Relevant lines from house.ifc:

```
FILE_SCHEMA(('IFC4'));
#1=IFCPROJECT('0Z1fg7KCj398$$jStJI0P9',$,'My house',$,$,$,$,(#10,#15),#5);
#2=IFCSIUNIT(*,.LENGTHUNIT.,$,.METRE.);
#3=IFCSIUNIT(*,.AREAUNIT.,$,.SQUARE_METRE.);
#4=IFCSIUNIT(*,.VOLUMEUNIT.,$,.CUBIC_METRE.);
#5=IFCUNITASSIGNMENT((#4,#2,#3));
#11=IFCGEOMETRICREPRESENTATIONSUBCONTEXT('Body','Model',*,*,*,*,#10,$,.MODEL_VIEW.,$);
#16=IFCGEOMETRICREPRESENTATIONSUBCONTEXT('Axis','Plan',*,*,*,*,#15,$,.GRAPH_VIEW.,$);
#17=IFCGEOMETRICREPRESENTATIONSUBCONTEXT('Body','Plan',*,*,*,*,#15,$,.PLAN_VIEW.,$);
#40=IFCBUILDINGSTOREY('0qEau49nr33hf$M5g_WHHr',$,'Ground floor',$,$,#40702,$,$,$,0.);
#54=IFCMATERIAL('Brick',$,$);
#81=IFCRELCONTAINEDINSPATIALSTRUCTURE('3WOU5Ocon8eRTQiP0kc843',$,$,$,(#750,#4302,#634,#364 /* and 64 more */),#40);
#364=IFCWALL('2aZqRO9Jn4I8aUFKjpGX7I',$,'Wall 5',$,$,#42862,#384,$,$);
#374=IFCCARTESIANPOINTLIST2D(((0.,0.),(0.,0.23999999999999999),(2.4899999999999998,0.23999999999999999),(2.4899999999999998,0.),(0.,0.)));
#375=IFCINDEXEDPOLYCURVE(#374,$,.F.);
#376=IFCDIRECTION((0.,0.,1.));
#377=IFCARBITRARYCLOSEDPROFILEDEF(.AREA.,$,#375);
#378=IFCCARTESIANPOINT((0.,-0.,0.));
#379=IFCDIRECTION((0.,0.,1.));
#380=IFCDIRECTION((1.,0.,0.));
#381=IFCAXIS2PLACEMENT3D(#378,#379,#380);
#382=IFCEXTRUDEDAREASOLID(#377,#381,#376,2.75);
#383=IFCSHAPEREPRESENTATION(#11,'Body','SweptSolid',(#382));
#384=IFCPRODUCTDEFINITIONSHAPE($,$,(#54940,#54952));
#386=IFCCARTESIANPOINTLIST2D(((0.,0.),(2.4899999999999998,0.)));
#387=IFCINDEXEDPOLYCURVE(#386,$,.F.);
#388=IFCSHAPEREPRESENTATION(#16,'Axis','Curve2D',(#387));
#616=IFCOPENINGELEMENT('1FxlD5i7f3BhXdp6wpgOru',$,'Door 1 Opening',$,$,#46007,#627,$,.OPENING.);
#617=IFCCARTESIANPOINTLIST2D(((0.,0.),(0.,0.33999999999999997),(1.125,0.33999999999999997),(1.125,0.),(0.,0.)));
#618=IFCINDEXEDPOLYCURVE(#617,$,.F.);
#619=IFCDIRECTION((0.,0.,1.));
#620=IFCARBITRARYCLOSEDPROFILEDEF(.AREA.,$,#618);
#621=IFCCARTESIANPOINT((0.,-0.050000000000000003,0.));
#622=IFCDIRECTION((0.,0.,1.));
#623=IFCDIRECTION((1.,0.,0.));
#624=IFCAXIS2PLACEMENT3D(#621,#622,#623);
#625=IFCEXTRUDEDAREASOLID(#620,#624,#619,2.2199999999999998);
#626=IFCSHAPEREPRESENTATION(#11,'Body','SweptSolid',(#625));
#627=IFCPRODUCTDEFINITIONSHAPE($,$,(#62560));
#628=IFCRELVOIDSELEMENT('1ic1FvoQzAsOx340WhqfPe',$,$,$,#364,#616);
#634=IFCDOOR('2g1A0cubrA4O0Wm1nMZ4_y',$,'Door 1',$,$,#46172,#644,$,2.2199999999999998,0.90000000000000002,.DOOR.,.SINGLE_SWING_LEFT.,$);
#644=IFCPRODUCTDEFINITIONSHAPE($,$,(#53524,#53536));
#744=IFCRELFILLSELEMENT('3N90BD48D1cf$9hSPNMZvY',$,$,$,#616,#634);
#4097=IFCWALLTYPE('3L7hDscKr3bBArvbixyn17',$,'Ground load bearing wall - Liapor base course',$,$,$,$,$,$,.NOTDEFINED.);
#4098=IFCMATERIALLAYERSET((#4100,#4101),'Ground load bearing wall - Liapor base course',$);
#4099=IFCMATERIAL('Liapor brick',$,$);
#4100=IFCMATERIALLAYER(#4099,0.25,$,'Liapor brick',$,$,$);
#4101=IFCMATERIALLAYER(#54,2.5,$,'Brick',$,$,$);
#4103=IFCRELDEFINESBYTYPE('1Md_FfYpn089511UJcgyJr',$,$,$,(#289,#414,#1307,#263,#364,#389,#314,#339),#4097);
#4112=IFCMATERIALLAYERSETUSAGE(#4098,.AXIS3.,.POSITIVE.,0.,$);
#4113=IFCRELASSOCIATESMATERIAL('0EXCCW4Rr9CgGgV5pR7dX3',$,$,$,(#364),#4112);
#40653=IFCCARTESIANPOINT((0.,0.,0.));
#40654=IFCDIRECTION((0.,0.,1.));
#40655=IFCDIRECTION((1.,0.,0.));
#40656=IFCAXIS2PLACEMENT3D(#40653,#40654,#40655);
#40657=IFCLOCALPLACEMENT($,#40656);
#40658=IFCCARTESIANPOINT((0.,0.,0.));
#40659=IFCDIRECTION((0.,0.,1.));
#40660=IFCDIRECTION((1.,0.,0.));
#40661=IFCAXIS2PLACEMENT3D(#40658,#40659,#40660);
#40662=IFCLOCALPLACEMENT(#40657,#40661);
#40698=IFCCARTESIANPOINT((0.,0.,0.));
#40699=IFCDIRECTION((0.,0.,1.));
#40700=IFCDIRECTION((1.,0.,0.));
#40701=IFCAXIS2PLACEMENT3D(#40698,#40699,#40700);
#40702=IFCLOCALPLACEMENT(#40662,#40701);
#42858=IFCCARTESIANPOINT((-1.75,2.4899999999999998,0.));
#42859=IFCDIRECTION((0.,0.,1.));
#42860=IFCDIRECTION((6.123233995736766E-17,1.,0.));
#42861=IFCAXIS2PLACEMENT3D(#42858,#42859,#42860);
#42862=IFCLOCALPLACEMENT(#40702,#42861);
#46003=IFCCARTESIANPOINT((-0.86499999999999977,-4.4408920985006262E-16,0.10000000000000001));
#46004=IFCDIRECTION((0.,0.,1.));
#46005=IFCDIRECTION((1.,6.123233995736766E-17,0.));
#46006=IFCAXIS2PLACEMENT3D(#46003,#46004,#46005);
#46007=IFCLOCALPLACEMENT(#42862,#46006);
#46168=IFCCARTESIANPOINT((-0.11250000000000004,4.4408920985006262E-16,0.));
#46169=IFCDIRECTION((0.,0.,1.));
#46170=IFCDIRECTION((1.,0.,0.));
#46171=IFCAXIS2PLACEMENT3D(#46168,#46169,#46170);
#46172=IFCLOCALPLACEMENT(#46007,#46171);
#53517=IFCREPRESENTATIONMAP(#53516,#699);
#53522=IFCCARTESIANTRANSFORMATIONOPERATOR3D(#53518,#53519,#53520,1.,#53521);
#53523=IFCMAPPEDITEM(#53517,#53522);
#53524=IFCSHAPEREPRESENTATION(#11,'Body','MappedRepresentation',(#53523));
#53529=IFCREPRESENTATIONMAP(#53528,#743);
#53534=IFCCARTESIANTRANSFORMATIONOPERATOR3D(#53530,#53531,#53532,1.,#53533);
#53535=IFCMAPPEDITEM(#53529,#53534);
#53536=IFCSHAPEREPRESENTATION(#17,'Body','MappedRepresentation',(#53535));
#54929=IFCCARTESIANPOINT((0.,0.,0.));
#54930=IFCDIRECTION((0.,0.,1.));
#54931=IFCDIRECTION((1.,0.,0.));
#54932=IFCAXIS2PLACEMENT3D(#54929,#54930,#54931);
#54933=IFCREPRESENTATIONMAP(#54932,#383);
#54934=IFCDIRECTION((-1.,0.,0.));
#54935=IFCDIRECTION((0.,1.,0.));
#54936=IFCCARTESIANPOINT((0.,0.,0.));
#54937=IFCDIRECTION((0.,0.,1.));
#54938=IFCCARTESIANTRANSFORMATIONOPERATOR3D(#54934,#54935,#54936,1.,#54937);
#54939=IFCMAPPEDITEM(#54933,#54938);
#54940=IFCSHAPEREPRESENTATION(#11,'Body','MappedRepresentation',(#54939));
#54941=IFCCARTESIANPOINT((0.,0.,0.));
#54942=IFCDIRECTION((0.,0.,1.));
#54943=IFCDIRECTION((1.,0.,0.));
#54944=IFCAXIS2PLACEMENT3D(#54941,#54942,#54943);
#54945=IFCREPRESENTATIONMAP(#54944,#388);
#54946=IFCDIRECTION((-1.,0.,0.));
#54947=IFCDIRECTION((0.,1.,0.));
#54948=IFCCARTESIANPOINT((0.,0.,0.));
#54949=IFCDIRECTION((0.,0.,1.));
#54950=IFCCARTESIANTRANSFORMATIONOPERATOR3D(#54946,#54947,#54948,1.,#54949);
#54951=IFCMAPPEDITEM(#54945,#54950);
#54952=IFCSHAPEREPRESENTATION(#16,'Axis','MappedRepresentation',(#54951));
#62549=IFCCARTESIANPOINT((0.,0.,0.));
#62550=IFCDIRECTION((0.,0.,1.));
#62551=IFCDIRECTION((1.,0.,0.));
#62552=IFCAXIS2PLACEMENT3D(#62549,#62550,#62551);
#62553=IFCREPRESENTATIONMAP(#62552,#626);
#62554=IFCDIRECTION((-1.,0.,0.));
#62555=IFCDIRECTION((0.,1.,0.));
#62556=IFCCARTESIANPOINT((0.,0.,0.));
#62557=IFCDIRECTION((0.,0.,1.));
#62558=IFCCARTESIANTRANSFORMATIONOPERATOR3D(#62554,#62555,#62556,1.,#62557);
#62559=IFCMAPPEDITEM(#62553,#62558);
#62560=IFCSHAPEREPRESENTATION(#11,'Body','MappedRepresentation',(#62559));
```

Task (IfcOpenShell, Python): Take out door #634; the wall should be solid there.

```python
import ifcopenshell
import ifcopenshell.api.feature
import ifcopenshell.api.root
import ifcopenshell.geom
import ifcopenshell.util.shape

model = ifcopenshell.open("house.ifc")
settings = ifcopenshell.geom.settings()


def volume(element):
    """Net volume in cubic metres, openings subtracted."""
    shape = ifcopenshell.geom.create_shape(settings, element)
    return ifcopenshell.util.shape.get_volume(shape.geometry)


door = model.by_guid("2g1A0cubrA4O0Wm1nMZ4_y")
opening = door.FillsVoids[0].RelatingOpeningElement
wall = opening.VoidsElements[0].RelatingBuildingElement
before = volume(wall)

ifcopenshell.api.root.remove_product(model, product=door)
ifcopenshell.api.feature.remove_feature(model, feature=opening)

after = volume(wall)

print(f"wall volume {before:.3f} -> {after:.3f} m3")

model.write("house_rev.ifc")
```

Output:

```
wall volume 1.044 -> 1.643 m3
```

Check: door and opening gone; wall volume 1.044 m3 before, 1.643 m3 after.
